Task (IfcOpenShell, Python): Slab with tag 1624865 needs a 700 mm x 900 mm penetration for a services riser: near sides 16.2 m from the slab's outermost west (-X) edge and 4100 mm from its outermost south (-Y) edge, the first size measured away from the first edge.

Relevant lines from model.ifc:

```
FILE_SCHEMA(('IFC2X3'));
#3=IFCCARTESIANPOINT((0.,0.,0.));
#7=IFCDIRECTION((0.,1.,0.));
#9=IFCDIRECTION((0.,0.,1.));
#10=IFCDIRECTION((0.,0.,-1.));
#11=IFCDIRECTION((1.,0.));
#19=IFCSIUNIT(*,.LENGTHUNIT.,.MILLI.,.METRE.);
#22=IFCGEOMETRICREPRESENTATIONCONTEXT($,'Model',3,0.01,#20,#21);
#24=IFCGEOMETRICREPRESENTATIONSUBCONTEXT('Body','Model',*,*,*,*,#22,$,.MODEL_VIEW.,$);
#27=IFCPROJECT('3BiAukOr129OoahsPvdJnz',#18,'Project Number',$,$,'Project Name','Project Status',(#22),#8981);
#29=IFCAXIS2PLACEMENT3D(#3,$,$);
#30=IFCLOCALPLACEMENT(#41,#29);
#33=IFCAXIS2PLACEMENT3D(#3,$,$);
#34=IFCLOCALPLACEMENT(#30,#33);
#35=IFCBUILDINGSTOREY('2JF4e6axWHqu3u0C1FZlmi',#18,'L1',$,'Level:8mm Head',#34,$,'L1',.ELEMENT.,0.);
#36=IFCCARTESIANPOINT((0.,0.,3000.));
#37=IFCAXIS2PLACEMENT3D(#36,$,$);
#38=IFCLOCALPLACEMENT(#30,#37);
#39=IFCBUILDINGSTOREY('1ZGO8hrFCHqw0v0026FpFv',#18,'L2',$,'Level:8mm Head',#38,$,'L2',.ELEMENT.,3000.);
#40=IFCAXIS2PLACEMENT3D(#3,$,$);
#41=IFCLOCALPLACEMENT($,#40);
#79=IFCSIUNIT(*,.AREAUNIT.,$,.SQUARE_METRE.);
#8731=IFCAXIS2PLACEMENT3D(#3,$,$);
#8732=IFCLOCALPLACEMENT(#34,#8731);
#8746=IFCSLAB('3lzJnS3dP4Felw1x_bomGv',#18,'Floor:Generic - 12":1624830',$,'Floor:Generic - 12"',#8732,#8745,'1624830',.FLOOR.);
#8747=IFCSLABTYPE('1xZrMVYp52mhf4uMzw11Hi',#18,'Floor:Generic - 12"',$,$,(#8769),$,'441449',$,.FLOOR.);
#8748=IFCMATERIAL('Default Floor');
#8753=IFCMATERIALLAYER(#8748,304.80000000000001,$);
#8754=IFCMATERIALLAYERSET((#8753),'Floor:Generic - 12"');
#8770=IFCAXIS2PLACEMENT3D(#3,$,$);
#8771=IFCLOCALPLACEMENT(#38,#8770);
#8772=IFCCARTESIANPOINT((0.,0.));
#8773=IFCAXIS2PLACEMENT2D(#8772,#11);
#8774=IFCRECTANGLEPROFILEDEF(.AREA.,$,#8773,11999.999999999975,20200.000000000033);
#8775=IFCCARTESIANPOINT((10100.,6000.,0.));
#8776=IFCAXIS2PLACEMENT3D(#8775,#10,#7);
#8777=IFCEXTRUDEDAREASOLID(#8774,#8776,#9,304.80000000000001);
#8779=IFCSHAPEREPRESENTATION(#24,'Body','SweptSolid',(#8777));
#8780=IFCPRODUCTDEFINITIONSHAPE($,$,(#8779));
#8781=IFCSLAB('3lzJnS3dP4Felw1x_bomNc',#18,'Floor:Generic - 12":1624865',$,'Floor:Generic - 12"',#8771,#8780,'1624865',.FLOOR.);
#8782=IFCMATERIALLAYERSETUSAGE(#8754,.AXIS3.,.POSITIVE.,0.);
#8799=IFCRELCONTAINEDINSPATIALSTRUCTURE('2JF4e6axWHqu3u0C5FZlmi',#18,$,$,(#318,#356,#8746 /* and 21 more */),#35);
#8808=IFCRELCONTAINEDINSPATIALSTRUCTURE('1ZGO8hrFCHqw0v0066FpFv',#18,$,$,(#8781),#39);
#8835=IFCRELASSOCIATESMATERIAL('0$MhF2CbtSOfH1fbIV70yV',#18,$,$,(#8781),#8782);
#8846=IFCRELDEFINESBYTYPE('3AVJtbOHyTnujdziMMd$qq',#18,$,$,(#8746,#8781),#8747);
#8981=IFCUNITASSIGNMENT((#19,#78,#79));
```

```python
import numpy as np
import ifcopenshell
import ifcopenshell.api.feature
import ifcopenshell.api.geometry
import ifcopenshell.api.root
import ifcopenshell.geom
import ifcopenshell.util.placement
import ifcopenshell.util.representation
import ifcopenshell.util.shape
import ifcopenshell.util.unit

model = ifcopenshell.open("model.ifc")
unit_scale = ifcopenshell.util.unit.calculate_unit_scale(model)
settings = ifcopenshell.geom.settings()


def volume(element):
    """Net volume in cubic metres, openings subtracted."""
    shape = ifcopenshell.geom.create_shape(settings, element)
    return ifcopenshell.util.shape.get_volume(shape.geometry)


slab = model.by_guid("3lzJnS3dP4Felw1x_bomNc")
before = volume(slab)

# Extent in the slab's own axes, in metres. The edges named are its -X and -Y sides.
slab_shape = ifcopenshell.geom.create_shape(settings, slab)
vertices = ifcopenshell.util.shape.get_vertices(slab_shape.geometry)
x_min, y_min, bottom = vertices.min(axis=0)
top = vertices[:, 2].max()

opening = ifcopenshell.api.root.create_entity(model, ifc_class="IfcOpeningElement", name="Services riser opening")
context = ifcopenshell.util.representation.get_context(model, "Model", "Body", "MODEL_VIEW")
width, depth = 0.7, 0.9
outline = [(0.0, 0.0), (width, 0.0), (width, depth), (0.0, depth), (0.0, 0.0)]
# Overshoot both faces by 50 mm so the cut is clean.
shape = ifcopenshell.api.geometry.add_slab_representation(
    model, context=context, depth=top - bottom + 0.1, polyline=outline
)
ifcopenshell.api.geometry.assign_representation(model, product=opening, representation=shape)

matrix = ifcopenshell.util.placement.get_local_placement(slab.ObjectPlacement)
matrix[:, 3] = matrix @ np.append(np.array([x_min + 16.2, y_min + 4.1, bottom - 0.05]) / unit_scale, 1.0)
ifcopenshell.api.geometry.edit_object_placement(model, product=opening, matrix=matrix, is_si=False)
ifcopenshell.api.feature.add_feature(model, feature=opening, element=slab)

after = volume(slab)

print(f"slab volume {before:.3f} -> {after:.3f} m3")

model.write("model_updated.ifc")
```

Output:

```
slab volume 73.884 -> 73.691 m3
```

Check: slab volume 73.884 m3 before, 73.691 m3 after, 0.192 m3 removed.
